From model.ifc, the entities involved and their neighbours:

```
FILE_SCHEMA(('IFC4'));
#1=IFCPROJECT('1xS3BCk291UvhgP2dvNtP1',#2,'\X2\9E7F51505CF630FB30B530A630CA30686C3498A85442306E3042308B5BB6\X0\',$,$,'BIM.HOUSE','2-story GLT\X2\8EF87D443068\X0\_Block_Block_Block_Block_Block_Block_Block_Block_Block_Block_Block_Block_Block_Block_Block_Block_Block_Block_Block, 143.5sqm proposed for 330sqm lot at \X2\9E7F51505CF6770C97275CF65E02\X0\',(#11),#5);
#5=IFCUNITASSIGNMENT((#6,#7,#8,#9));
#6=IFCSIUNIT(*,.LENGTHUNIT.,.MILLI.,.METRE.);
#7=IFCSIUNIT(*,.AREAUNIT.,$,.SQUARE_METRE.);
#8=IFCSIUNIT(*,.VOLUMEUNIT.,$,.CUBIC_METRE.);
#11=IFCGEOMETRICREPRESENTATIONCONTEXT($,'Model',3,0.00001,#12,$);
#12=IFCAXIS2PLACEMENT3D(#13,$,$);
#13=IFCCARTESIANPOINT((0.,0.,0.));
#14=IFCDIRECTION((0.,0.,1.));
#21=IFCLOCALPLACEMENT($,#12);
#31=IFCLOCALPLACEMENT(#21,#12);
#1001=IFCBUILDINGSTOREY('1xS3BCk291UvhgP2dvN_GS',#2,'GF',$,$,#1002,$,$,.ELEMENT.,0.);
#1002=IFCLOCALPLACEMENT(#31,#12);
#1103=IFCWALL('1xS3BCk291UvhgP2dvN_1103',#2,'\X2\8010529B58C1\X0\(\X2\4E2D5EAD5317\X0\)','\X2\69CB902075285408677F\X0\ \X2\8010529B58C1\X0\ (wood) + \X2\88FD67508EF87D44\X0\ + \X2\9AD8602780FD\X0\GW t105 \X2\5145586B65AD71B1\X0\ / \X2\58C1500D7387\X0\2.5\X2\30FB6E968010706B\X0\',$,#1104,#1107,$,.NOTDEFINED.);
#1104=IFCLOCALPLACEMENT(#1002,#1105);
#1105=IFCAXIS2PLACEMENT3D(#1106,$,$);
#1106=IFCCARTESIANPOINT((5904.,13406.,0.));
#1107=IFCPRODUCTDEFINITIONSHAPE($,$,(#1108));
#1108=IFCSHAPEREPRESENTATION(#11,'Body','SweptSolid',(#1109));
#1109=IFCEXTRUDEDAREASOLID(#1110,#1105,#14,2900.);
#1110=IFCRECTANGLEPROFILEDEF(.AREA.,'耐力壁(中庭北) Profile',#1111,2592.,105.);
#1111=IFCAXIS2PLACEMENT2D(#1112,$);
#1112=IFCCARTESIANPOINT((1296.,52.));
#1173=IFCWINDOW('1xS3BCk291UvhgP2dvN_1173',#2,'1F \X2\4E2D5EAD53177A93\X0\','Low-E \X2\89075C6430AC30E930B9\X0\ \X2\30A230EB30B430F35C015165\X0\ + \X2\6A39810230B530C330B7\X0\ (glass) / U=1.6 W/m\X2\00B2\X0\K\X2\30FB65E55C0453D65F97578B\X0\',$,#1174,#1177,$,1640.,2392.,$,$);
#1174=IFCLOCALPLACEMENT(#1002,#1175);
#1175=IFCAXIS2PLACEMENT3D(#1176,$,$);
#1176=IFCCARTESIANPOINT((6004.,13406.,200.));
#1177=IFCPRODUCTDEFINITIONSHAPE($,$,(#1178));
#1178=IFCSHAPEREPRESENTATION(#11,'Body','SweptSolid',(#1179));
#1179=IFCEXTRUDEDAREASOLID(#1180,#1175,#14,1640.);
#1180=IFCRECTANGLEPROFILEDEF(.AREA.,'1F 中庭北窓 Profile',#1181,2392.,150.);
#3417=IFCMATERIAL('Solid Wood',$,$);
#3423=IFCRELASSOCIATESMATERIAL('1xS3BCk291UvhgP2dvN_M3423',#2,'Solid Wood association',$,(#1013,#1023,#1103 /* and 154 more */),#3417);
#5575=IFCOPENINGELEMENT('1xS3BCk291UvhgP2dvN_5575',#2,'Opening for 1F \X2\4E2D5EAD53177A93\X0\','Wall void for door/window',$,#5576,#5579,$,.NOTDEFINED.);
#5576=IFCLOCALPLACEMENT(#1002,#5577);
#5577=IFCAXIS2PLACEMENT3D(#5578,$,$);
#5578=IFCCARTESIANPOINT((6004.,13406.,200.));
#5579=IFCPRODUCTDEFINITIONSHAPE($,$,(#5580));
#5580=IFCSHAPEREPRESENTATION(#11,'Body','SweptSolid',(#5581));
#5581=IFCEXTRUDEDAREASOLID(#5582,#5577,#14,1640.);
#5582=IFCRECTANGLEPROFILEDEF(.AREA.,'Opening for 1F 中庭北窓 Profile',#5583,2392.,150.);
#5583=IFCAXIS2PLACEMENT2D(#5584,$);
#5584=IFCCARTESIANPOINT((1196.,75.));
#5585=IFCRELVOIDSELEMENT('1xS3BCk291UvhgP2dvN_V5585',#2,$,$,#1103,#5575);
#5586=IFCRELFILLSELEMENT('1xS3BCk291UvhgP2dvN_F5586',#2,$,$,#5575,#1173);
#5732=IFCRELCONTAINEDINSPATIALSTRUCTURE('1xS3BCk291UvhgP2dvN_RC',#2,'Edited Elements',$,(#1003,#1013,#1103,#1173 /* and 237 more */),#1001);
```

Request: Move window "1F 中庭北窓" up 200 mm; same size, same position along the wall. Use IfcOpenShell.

```python
import numpy as np
import ifcopenshell
import ifcopenshell.api.geometry
import ifcopenshell.util.placement
import ifcopenshell.util.unit

model = ifcopenshell.open("model.ifc")
unit_scale = ifcopenshell.util.unit.calculate_unit_scale(model)

window = model.by_guid("1xS3BCk291UvhgP2dvN_1173")
opening = window.FillsVoids[0].RelatingOpeningElement
dz = 0.2 / unit_scale

shift = np.array([0.0, 0.0, dz])
# The window is not placed relative to its opening, so move both.
for product in (opening, window):
    matrix = ifcopenshell.util.placement.get_local_placement(product.ObjectPlacement)
    matrix[:3, 3] += shift
    ifcopenshell.api.geometry.edit_object_placement(model, product=product, matrix=matrix, is_si=False)

print(f"moved by {dz * unit_scale:+.3f} m")

model.write("model_v2.ifc")
```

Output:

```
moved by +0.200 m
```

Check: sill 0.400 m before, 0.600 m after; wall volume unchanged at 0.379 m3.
